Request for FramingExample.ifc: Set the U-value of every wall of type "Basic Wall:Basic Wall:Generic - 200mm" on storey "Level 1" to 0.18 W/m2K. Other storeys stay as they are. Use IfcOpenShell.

First a look at what the model holds.

```python
import ifcopenshell
import ifcopenshell.util.element

model = ifcopenshell.open("FramingExample.ifc")
print(model.schema)
storey = next(s for s in model.by_type("IfcBuildingStorey") if s.Name == "Level 1")
walls = [e for e in ifcopenshell.util.element.get_decomposition(storey) if e.is_a("IfcWall")]
seen = {}
for e in walls:
    element_type = ifcopenshell.util.element.get_type(e)
    key = (element_type.Name if element_type != e and element_type else None, ifcopenshell.util.element.get_pset(e, "Pset_WallCommon", "ThermalTransmittance"))
    seen[key] = seen.get(key, 0) + 1
for (name, value), count in sorted(seen.items(), key=str):
    print(count, "x", name, "|", value)
```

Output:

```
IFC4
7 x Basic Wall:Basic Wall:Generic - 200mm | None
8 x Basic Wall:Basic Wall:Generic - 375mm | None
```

```python
import ifcopenshell
import ifcopenshell.api.pset
import ifcopenshell.util.element

model = ifcopenshell.open("FramingExample.ifc")

storey = next(s for s in model.by_type("IfcBuildingStorey") if s.Name == "Level 1")
walls = [e for e in ifcopenshell.util.element.get_decomposition(storey) if e.is_a("IfcWall")]

count = 0
for e in walls:
    element_type = ifcopenshell.util.element.get_type(e)
    if element_type in (None, e) or element_type.Name != "Basic Wall:Basic Wall:Generic - 200mm":
        continue
    # add_pset returns the element's existing set when there is one.
    pset = ifcopenshell.api.pset.add_pset(model, product=e, name="Pset_WallCommon")
    ifcopenshell.api.pset.edit_pset(model, pset=pset, properties={"ThermalTransmittance": 0.18})
    count += 1

print(count, "walls updated")

model.write("FramingExample-out.ifc")
```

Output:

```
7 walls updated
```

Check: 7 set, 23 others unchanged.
